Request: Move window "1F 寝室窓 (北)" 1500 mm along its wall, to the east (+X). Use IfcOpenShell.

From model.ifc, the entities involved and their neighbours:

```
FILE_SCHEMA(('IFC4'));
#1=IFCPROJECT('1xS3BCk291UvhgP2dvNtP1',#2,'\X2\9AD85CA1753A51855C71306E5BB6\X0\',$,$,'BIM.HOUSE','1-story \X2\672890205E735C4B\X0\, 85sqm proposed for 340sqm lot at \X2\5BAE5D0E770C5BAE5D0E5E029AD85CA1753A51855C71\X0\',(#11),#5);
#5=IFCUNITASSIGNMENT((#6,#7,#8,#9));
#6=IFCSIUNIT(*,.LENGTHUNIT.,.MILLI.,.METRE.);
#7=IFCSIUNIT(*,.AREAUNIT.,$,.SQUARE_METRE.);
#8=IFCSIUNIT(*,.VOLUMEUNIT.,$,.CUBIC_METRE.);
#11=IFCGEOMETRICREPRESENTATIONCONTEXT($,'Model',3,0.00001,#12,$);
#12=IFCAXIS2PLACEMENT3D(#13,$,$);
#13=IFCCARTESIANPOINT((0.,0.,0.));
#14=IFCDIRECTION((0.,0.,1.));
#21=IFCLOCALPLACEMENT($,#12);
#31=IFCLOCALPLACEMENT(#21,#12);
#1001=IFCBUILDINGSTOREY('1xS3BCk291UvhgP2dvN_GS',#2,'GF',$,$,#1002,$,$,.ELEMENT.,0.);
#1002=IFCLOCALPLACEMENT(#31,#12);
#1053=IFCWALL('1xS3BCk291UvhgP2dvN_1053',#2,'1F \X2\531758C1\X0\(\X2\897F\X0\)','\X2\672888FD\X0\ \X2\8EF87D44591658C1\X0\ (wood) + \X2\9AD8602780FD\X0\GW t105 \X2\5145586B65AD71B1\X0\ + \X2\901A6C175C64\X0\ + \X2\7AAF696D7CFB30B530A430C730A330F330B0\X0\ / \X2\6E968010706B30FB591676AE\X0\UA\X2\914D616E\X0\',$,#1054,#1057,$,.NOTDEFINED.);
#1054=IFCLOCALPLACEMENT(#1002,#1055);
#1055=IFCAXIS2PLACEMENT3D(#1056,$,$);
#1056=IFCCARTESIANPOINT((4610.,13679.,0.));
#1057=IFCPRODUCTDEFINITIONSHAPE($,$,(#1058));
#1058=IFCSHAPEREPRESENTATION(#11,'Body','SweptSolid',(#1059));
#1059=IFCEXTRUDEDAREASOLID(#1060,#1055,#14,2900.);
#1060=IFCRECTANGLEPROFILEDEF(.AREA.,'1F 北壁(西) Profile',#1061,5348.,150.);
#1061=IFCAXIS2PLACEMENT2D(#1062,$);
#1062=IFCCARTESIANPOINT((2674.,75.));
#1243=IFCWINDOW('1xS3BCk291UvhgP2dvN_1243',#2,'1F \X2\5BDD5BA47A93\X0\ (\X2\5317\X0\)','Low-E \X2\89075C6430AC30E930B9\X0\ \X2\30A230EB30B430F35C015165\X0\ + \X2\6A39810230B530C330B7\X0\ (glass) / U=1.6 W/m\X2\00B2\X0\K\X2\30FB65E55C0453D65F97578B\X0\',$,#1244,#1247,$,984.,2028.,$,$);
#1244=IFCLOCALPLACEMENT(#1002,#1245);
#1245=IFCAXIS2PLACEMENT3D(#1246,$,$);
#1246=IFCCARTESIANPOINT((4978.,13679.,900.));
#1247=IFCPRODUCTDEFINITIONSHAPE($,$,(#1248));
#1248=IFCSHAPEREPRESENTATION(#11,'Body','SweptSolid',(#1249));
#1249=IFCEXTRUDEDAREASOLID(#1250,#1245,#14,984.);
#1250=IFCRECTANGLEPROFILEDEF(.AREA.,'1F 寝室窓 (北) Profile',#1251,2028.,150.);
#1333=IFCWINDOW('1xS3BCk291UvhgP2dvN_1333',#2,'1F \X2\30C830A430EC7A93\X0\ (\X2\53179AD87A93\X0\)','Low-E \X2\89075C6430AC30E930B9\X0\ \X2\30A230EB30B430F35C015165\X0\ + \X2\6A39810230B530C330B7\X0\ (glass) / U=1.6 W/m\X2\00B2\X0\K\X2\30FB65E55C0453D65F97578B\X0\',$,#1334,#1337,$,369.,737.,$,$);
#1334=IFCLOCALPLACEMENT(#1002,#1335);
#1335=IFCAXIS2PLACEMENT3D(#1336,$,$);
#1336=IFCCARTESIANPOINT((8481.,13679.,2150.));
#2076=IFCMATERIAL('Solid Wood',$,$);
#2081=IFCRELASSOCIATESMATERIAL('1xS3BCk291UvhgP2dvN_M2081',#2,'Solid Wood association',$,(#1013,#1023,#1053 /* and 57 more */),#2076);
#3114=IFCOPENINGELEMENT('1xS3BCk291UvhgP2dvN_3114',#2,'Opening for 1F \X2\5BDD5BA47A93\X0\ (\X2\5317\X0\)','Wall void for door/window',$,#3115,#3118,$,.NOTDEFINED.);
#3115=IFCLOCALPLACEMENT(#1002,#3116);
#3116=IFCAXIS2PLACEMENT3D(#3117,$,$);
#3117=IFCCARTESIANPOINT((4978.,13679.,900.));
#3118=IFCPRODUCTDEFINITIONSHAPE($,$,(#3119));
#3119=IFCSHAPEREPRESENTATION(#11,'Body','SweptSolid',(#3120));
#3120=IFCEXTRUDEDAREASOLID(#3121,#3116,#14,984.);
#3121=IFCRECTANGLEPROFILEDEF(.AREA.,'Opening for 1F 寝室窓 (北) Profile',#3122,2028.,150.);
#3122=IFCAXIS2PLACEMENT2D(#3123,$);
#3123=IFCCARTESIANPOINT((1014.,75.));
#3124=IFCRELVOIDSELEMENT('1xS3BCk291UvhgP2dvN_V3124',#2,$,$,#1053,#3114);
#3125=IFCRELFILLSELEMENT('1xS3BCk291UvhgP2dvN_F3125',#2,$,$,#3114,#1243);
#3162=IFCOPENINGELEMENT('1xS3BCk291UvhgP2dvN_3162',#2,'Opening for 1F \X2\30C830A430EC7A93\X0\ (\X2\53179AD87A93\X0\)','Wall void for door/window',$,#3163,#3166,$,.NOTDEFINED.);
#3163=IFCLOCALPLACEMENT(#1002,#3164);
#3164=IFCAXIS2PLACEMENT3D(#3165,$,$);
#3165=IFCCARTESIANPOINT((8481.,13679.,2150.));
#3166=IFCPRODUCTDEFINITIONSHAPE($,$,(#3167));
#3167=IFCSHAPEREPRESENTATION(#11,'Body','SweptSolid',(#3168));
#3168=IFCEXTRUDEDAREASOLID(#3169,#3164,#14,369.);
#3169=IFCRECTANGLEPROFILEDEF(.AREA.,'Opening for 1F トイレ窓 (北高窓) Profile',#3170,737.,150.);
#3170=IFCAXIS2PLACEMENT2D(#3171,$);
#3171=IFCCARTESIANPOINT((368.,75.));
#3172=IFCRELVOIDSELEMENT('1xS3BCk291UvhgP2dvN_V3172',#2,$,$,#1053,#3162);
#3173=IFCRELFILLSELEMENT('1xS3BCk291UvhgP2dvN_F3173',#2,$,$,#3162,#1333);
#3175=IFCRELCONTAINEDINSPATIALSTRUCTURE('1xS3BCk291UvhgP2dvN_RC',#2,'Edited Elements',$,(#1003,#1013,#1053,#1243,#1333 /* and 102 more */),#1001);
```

```python
import ifcopenshell
import ifcopenshell.api.geometry
import ifcopenshell.util.placement

model = ifcopenshell.open("model.ifc")

window = model.by_guid("1xS3BCk291UvhgP2dvN_1243")
opening = window.FillsVoids[0].RelatingOpeningElement
wall = opening.VoidsElements[0].RelatingBuildingElement

wall_matrix = ifcopenshell.util.placement.get_local_placement(wall.ObjectPlacement)
shift = wall_matrix[:3, 0] * 1500.0
before = ifcopenshell.util.placement.get_local_placement(window.ObjectPlacement)[:3, 3].copy()

# The window is not placed relative to its opening, so move both.
for product in (opening, window):
    matrix = ifcopenshell.util.placement.get_local_placement(product.ObjectPlacement)
    matrix[:3, 3] += shift
    ifcopenshell.api.geometry.edit_object_placement(model, product=product, matrix=matrix, is_si=False)

after = ifcopenshell.util.placement.get_local_placement(window.ObjectPlacement)[:3, 3]
print("window moved by", (after - before).round(3) + 0.0)

model.write("model_rev.ifc")
```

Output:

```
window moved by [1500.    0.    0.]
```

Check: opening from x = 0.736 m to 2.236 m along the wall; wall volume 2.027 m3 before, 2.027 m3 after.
